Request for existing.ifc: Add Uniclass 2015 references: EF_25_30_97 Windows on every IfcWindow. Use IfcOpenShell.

First a look at what the model holds.

```python
import ifcopenshell

model = ifcopenshell.open("existing.ifc")
print(model.schema)
print("classifications:", [c.Name for c in model.by_type("IfcClassification")])
for ifc_class in ("IfcDoor", "IfcRoof", "IfcStair", "IfcWall", "IfcWindow"):
    print(ifc_class, len(model.by_type(ifc_class)))
```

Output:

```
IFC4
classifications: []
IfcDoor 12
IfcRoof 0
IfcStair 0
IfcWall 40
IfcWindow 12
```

```python
import ifcopenshell
import ifcopenshell.api.classification

model = ifcopenshell.open("existing.ifc")

system = ifcopenshell.api.classification.add_classification(model, classification="Uniclass 2015")

codes = {
    "IfcWindow": ("EF_25_30_97", "Windows"),
}
for ifc_class, (code, name) in codes.items():
    products = model.by_type(ifc_class)
    ifcopenshell.api.classification.add_reference(
        model, products=products, classification=system, identification=code, name=name
    )
    print(code, len(products))

model.write("existing-out.ifc")
```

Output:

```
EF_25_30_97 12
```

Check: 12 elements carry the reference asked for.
